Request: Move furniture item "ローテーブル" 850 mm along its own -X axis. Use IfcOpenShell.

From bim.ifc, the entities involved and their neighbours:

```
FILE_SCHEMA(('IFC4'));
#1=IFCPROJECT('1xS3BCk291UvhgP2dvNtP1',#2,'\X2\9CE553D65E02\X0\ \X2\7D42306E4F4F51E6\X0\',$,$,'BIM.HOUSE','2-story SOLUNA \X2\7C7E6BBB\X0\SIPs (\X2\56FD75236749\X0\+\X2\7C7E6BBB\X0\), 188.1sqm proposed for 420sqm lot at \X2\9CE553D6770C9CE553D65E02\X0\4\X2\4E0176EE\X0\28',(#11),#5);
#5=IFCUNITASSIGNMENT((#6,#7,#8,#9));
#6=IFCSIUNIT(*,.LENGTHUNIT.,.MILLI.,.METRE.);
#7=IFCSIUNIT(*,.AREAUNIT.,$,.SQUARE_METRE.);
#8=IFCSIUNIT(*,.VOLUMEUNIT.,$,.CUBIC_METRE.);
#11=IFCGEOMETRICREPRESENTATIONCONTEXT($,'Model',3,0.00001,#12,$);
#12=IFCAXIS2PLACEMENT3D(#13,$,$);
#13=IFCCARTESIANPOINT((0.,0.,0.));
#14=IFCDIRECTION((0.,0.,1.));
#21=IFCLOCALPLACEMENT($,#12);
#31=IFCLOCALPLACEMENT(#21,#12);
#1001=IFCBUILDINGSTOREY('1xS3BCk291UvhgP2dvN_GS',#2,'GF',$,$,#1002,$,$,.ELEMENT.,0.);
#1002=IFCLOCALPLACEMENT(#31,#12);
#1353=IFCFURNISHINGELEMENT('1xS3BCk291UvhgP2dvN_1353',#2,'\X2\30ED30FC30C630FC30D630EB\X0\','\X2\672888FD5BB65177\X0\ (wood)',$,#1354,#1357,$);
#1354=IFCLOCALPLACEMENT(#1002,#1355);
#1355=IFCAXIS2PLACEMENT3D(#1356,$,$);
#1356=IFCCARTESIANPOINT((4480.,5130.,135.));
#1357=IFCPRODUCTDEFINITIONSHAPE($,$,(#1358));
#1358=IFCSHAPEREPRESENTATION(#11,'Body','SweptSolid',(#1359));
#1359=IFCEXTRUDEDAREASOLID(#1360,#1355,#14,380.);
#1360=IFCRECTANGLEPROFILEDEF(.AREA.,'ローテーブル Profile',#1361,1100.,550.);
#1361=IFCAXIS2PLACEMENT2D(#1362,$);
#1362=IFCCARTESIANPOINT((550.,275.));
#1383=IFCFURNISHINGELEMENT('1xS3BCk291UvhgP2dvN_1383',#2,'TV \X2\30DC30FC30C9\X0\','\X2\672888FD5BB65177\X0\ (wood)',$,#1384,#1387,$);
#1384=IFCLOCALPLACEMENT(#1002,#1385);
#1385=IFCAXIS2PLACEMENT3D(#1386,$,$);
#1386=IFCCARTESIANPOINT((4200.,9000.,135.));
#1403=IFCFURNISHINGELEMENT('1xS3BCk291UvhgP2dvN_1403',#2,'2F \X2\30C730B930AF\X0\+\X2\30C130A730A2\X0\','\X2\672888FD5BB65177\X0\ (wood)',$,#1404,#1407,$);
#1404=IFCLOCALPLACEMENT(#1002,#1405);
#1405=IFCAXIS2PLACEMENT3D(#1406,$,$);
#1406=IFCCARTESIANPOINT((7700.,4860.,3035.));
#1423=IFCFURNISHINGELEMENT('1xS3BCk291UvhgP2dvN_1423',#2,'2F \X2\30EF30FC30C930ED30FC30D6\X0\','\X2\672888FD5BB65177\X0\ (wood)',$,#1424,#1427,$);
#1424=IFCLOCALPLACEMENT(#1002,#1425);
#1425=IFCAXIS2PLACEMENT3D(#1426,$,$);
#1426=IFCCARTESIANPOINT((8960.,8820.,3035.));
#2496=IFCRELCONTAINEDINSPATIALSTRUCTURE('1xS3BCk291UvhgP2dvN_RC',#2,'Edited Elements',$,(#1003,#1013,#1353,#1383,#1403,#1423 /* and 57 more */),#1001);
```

```python
import ifcopenshell
import ifcopenshell.api.geometry
import ifcopenshell.util.placement
import ifcopenshell.util.unit

model = ifcopenshell.open("bim.ifc")
unit_scale = ifcopenshell.util.unit.calculate_unit_scale(model)

item = model.by_guid("1xS3BCk291UvhgP2dvN_1353")
matrix = ifcopenshell.util.placement.get_local_placement(item.ObjectPlacement)
matrix[:3, 3] -= matrix[:3, 0] * 0.85 / unit_scale
ifcopenshell.api.geometry.edit_object_placement(model, product=item, matrix=matrix, is_si=False)

print(ifcopenshell.util.placement.get_local_placement(item.ObjectPlacement).round(3) + 0.0)

model.write("bim_v2.ifc")
```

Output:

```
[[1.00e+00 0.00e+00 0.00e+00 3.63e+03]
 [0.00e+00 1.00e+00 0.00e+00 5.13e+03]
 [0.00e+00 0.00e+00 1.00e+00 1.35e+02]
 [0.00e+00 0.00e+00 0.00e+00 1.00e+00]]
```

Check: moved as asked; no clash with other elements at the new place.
